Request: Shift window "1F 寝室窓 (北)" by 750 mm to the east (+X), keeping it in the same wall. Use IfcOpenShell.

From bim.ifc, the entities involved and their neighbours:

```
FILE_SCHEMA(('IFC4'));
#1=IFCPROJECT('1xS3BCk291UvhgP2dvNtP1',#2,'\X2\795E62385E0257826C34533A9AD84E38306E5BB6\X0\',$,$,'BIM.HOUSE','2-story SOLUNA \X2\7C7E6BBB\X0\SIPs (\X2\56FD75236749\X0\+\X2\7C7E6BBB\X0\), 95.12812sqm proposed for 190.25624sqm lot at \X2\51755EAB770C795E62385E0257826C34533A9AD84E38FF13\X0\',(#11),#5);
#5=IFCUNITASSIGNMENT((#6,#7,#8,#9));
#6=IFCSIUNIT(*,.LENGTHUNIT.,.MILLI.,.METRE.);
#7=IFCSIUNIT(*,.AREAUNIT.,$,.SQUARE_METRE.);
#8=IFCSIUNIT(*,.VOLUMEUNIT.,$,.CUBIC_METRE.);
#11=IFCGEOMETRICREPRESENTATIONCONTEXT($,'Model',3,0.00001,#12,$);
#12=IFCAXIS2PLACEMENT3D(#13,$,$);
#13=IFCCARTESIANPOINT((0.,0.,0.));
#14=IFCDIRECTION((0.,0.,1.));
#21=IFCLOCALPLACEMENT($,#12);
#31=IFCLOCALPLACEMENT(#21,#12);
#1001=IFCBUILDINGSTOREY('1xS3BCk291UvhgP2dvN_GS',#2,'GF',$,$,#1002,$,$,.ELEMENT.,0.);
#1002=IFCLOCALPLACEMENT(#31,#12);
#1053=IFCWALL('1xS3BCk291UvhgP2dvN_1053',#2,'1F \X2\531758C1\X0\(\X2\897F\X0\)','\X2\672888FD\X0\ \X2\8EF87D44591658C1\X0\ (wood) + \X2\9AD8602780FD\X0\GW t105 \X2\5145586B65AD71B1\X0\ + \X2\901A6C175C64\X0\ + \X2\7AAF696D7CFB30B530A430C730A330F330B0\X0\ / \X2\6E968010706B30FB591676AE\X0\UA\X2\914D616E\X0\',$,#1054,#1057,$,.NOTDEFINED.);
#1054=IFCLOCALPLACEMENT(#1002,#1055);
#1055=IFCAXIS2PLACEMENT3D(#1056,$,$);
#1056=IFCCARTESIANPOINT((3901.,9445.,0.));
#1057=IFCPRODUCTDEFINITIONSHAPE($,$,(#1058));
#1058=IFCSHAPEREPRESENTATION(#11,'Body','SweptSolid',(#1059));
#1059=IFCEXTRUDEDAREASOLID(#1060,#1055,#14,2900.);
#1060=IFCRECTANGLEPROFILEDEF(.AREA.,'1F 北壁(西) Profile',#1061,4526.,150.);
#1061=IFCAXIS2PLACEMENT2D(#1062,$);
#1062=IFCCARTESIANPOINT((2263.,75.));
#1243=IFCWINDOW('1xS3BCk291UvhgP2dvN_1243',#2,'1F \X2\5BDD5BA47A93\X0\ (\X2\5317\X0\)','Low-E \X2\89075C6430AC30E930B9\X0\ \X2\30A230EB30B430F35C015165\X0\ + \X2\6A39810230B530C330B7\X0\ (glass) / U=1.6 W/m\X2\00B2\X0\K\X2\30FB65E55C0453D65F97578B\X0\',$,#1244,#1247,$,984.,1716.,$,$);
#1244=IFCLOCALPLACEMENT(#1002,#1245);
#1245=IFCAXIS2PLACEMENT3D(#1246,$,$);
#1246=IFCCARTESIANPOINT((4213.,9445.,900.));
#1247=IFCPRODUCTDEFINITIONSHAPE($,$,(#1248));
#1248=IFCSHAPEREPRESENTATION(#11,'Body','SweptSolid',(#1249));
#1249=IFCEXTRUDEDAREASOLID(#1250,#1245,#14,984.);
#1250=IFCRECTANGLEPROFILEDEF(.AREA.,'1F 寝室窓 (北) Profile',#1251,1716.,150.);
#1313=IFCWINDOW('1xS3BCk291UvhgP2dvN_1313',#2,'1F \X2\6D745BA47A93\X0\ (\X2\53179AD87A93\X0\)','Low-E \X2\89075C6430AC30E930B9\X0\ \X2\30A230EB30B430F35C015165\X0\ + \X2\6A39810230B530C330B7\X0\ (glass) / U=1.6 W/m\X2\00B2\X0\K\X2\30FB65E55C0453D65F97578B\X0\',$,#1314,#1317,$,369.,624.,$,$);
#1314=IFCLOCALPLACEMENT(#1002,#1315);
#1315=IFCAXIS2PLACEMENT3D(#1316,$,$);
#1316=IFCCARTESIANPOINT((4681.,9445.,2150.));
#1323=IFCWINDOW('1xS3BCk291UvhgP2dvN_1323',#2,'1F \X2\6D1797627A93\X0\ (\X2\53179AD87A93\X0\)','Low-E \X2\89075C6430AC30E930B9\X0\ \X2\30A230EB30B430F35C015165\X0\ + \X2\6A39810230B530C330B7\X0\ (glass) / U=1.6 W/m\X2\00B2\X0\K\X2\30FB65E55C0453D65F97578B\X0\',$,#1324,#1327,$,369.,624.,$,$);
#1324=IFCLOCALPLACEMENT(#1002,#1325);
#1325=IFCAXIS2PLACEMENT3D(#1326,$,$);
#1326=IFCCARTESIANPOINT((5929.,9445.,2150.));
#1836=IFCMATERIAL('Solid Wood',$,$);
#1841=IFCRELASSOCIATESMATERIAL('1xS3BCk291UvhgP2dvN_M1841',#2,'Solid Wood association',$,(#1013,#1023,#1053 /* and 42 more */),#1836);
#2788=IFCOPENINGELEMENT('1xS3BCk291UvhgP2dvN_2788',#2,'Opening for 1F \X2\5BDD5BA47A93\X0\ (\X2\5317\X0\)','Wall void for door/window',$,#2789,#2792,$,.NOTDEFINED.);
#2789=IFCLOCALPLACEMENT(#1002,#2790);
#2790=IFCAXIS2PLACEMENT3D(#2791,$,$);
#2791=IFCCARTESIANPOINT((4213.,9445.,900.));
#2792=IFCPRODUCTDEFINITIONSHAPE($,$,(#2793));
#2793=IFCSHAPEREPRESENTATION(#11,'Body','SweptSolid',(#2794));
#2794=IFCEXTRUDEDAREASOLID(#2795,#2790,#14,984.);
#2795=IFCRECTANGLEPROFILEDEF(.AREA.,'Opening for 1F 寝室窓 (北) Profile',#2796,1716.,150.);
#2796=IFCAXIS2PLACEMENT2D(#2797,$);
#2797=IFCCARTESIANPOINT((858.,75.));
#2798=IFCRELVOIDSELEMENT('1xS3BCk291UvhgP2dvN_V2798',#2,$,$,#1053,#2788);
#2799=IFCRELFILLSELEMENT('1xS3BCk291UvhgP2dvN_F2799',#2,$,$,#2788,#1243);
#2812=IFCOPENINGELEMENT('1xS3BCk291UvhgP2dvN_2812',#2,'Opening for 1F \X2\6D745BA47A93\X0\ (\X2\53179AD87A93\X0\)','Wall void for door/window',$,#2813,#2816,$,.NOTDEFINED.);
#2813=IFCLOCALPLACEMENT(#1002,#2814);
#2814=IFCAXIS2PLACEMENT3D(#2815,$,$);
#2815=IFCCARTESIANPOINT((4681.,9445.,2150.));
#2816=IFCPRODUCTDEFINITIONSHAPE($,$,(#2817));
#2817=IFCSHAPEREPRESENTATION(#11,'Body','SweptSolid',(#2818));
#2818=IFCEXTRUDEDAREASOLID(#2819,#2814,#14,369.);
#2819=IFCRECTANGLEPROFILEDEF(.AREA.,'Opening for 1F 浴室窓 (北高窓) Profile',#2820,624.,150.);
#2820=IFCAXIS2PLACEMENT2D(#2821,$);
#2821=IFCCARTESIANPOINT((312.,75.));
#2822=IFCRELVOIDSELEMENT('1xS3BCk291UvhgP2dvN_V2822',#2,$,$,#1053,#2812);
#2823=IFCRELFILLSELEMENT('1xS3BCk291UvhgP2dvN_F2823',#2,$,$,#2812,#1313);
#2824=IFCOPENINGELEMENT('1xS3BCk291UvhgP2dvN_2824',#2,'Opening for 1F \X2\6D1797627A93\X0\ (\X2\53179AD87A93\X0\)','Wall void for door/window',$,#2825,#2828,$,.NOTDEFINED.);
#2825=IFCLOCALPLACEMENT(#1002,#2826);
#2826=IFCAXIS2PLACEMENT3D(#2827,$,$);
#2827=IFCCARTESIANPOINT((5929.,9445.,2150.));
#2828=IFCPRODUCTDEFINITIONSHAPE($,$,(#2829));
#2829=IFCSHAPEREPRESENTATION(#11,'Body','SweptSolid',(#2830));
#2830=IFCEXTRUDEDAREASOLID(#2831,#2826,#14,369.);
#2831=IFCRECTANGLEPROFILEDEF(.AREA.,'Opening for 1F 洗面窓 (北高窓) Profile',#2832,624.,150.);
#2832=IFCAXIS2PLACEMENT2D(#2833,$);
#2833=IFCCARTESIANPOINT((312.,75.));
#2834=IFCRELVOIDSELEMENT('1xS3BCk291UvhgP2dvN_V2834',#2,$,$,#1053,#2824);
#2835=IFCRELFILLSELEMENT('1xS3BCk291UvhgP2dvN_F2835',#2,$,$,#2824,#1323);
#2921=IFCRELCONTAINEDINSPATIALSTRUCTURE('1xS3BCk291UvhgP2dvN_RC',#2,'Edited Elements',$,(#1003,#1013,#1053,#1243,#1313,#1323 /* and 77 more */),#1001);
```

```python
import ifcopenshell
import ifcopenshell.api.geometry
import ifcopenshell.util.placement

model = ifcopenshell.open("bim.ifc")

window = model.by_guid("1xS3BCk291UvhgP2dvN_1243")
opening = window.FillsVoids[0].RelatingOpeningElement
wall = opening.VoidsElements[0].RelatingBuildingElement

wall_matrix = ifcopenshell.util.placement.get_local_placement(wall.ObjectPlacement)
shift = wall_matrix[:3, 0] * 750.0
before = ifcopenshell.util.placement.get_local_placement(window.ObjectPlacement)[:3, 3].copy()

# The window is not placed relative to its opening, so move both.
for product in (opening, window):
    matrix = ifcopenshell.util.placement.get_local_placement(product.ObjectPlacement)
    matrix[:3, 3] += shift
    ifcopenshell.api.geometry.edit_object_placement(model, product=product, matrix=matrix, is_si=False)

after = ifcopenshell.util.placement.get_local_placement(window.ObjectPlacement)[:3, 3]
print("window moved by", (after - before).round(3) + 0.0)

model.write("bim_rev.ifc")
```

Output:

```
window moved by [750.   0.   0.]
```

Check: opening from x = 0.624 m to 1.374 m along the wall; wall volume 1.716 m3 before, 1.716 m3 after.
